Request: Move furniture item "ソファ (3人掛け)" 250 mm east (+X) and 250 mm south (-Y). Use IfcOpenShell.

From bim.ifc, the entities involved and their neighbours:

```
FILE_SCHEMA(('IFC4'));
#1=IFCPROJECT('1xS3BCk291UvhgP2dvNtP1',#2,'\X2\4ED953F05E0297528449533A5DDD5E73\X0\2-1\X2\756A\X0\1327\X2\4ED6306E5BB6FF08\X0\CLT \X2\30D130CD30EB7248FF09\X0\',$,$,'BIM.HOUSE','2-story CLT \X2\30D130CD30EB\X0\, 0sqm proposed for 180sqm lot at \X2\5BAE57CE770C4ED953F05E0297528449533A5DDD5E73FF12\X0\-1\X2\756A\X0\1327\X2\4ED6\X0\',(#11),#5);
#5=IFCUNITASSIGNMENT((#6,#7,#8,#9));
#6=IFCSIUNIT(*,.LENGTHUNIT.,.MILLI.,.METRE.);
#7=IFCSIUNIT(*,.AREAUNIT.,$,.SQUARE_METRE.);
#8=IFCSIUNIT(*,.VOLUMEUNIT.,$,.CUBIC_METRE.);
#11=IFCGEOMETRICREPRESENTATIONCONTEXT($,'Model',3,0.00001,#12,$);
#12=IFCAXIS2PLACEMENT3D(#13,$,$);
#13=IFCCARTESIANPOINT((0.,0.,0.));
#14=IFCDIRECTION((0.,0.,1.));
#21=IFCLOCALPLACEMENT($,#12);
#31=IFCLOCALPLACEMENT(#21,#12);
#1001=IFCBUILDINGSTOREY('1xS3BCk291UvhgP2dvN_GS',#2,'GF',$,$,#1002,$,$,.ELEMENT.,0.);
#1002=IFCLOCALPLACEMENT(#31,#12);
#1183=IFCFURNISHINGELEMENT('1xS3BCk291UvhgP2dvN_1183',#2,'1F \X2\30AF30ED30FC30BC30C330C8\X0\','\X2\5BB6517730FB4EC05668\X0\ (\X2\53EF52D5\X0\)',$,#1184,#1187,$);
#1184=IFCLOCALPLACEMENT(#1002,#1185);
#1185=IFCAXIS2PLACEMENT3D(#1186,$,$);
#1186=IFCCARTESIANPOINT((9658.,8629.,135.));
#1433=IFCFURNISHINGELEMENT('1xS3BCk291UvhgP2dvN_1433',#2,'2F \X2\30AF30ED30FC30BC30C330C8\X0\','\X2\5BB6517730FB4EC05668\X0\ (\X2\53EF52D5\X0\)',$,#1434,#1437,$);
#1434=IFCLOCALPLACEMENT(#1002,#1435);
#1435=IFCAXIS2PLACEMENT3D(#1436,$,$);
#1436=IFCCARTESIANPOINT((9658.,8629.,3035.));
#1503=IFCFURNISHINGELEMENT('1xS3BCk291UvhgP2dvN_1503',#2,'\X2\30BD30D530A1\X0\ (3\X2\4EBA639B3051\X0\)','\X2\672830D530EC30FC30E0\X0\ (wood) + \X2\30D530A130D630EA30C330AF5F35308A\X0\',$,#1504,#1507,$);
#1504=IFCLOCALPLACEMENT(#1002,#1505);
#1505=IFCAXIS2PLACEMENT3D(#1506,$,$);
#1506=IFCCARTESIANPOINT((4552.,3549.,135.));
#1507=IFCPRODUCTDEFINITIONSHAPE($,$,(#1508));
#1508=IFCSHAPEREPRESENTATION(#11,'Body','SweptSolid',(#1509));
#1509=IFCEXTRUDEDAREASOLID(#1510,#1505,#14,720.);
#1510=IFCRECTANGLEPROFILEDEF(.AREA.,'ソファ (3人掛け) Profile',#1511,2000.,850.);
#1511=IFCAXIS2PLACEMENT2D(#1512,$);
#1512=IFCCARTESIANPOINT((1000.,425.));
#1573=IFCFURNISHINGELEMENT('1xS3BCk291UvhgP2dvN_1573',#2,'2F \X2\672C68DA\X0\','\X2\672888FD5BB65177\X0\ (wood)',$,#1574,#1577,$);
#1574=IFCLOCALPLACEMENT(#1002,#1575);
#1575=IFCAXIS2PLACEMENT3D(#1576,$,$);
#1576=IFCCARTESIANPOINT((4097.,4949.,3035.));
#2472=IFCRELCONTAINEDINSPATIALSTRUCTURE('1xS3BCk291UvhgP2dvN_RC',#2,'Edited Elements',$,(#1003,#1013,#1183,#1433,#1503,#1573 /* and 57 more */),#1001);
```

```python
import ifcopenshell
import ifcopenshell.api.geometry
import ifcopenshell.util.placement

model = ifcopenshell.open("bim.ifc")

item = model.by_guid("1xS3BCk291UvhgP2dvN_1503")
matrix = ifcopenshell.util.placement.get_local_placement(item.ObjectPlacement)
matrix[0, 3] += 250.0
matrix[1, 3] -= 250.0
ifcopenshell.api.geometry.edit_object_placement(model, product=item, matrix=matrix, is_si=False)

print(ifcopenshell.util.placement.get_local_placement(item.ObjectPlacement).round(3) + 0.0)

model.write("bim_rev.ifc")
```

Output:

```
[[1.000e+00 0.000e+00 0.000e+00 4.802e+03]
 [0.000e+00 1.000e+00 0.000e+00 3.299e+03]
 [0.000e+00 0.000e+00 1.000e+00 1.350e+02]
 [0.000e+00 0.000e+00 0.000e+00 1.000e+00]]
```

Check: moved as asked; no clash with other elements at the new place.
